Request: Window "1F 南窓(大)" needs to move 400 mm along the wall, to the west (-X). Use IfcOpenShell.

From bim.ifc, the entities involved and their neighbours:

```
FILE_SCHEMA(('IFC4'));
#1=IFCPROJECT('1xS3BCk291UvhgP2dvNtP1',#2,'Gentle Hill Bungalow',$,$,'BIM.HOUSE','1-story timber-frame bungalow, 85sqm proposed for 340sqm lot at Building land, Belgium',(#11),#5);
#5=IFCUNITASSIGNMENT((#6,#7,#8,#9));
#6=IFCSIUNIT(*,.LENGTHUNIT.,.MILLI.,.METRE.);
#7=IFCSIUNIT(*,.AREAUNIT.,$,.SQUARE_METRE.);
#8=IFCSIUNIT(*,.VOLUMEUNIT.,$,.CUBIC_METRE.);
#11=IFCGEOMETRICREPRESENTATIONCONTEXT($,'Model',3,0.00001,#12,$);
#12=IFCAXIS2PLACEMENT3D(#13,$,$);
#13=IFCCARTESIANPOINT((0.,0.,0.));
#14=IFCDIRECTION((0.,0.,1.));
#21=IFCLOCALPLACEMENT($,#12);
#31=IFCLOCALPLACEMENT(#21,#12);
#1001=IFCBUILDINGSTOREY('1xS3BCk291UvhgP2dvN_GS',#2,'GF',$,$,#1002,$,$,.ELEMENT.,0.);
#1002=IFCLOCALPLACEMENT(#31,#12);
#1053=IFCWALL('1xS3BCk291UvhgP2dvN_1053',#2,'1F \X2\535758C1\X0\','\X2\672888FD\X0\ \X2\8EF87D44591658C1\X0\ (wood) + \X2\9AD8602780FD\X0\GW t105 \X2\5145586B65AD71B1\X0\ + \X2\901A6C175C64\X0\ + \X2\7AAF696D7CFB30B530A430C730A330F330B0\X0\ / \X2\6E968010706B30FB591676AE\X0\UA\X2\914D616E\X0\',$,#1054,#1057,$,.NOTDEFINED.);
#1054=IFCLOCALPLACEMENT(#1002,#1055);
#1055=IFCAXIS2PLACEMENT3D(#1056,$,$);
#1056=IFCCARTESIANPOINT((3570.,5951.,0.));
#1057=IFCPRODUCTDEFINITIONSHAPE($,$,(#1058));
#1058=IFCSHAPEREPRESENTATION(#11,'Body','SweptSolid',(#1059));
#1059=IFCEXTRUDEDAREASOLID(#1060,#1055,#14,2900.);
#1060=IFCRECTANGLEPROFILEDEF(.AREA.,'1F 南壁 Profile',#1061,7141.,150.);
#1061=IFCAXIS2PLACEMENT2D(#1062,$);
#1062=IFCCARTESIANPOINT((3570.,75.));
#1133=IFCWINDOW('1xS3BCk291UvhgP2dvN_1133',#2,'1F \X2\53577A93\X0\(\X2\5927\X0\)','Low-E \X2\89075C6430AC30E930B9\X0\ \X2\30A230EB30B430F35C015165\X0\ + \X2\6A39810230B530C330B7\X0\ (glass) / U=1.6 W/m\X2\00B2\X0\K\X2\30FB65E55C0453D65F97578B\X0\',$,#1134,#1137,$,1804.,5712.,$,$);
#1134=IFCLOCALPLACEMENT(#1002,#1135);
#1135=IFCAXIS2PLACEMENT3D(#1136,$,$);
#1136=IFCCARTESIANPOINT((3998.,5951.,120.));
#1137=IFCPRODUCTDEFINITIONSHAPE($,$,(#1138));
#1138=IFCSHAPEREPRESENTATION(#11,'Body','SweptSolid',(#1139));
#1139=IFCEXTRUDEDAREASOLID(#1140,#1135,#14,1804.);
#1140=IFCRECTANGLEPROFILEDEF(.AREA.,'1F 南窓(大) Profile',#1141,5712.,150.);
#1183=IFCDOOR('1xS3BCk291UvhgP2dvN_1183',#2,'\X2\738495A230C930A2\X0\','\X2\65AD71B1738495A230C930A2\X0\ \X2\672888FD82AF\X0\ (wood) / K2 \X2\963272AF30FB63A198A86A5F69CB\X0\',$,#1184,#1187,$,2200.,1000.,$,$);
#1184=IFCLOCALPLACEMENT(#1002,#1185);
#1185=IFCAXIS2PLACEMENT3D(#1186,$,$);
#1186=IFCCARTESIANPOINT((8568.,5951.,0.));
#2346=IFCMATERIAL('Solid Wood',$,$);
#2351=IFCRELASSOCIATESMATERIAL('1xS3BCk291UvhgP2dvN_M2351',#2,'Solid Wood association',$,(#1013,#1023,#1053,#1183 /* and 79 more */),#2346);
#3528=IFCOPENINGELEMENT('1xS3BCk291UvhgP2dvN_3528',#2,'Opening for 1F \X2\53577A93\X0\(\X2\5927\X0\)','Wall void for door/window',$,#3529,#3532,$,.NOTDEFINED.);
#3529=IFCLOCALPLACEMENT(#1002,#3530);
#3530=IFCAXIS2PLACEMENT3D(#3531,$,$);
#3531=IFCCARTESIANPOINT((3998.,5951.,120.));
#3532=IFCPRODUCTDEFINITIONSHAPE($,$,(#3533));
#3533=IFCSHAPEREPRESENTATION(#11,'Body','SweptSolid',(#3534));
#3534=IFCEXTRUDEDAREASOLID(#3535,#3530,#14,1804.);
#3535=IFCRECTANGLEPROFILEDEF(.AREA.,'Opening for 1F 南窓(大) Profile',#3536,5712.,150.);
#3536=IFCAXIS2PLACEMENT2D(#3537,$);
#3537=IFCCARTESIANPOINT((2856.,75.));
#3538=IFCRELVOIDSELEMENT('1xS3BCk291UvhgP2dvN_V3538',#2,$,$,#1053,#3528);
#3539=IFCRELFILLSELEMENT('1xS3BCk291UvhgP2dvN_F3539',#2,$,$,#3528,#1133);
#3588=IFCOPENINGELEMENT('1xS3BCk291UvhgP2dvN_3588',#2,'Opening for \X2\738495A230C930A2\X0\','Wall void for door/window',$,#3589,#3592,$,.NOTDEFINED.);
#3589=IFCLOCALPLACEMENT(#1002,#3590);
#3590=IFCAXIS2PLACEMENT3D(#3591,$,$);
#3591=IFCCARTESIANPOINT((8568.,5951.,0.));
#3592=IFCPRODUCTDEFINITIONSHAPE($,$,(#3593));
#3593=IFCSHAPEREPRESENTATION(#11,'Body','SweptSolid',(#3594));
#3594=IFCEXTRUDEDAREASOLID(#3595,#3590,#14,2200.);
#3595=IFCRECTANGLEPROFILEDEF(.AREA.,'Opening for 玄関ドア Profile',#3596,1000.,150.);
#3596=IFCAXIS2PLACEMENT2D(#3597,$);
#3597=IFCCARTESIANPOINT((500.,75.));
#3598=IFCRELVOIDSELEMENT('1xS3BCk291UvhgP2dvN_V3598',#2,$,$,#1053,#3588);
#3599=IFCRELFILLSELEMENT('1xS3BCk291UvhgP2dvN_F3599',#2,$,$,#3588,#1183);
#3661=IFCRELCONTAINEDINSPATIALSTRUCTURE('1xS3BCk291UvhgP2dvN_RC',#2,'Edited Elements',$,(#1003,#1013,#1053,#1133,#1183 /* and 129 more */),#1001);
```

```python
import ifcopenshell
import ifcopenshell.api.geometry
import ifcopenshell.util.placement
import ifcopenshell.util.unit

model = ifcopenshell.open("bim.ifc")
unit_scale = ifcopenshell.util.unit.calculate_unit_scale(model)

window = model.by_guid("1xS3BCk291UvhgP2dvN_1133")
opening = window.FillsVoids[0].RelatingOpeningElement
wall = opening.VoidsElements[0].RelatingBuildingElement

wall_matrix = ifcopenshell.util.placement.get_local_placement(wall.ObjectPlacement)
shift = wall_matrix[:3, 0] * -0.4 / unit_scale
before = ifcopenshell.util.placement.get_local_placement(window.ObjectPlacement)[:3, 3].copy()

# The window is not placed relative to its opening, so move both.
for product in (opening, window):
    matrix = ifcopenshell.util.placement.get_local_placement(product.ObjectPlacement)
    matrix[:3, 3] += shift
    ifcopenshell.api.geometry.edit_object_placement(model, product=product, matrix=matrix, is_si=False)

after = ifcopenshell.util.placement.get_local_placement(window.ObjectPlacement)[:3, 3]
print("window moved by", (after - before).round(3) + 0.0)

model.write("bim_v2.ifc")
```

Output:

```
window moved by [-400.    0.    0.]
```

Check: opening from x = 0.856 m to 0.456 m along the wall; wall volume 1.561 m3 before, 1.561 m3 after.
